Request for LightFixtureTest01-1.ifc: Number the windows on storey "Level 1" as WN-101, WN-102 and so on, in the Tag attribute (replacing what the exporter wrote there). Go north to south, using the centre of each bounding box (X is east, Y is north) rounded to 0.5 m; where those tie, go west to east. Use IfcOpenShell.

First a look at what the model holds.

```python
import ifcopenshell
import ifcopenshell.util.element
import ifcopenshell.util.placement

model = ifcopenshell.open("LightFixtureTest01-1.ifc")
print(model.schema)
storey = next(s for s in model.by_type("IfcBuildingStorey") if s.Name == "Level 1")
windows = [e for e in ifcopenshell.util.element.get_decomposition(storey) if e.is_a("IfcWindow")]
for e in sorted(windows, key=lambda e: e.id()):
    origin = ifcopenshell.util.placement.get_local_placement(e.ObjectPlacement)[:3, 3]
    print(e.id(), e.Tag, e.Name, origin.round(2) + 0.0, sep=" | ")
```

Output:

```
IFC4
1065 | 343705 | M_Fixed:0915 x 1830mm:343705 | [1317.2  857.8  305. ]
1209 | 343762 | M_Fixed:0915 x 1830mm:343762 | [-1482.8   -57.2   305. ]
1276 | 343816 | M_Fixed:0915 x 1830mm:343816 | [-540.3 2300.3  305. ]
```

```python
import ifcopenshell
import ifcopenshell.geom
import ifcopenshell.util.element
import ifcopenshell.util.shape

model = ifcopenshell.open("LightFixtureTest01-1.ifc")
settings = ifcopenshell.geom.settings()
settings.set("use-world-coords", True)


def centre(element):
    shape = ifcopenshell.geom.create_shape(settings, element)
    return ifcopenshell.util.shape.get_bbox_centroid(shape.geometry)


storey = next(s for s in model.by_type("IfcBuildingStorey") if s.Name == "Level 1")
windows = [e for e in ifcopenshell.util.element.get_decomposition(storey) if e.is_a("IfcWindow")]

# Insertion points can sit at a corner or the storey origin, so sort by the geometry (in metres).
centres = {e: centre(e) for e in windows}
windows.sort(key=lambda e: (-round(centres[e][1] / 0.5), centres[e][0]))

for i, e in enumerate(windows, start=1):
    number = f"WN-1{i:02d}"
    e.Tag = number
    print(e.id(), number)

model.write("LightFixtureTest01-1-out.ifc")
```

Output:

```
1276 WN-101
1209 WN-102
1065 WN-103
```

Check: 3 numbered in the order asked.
